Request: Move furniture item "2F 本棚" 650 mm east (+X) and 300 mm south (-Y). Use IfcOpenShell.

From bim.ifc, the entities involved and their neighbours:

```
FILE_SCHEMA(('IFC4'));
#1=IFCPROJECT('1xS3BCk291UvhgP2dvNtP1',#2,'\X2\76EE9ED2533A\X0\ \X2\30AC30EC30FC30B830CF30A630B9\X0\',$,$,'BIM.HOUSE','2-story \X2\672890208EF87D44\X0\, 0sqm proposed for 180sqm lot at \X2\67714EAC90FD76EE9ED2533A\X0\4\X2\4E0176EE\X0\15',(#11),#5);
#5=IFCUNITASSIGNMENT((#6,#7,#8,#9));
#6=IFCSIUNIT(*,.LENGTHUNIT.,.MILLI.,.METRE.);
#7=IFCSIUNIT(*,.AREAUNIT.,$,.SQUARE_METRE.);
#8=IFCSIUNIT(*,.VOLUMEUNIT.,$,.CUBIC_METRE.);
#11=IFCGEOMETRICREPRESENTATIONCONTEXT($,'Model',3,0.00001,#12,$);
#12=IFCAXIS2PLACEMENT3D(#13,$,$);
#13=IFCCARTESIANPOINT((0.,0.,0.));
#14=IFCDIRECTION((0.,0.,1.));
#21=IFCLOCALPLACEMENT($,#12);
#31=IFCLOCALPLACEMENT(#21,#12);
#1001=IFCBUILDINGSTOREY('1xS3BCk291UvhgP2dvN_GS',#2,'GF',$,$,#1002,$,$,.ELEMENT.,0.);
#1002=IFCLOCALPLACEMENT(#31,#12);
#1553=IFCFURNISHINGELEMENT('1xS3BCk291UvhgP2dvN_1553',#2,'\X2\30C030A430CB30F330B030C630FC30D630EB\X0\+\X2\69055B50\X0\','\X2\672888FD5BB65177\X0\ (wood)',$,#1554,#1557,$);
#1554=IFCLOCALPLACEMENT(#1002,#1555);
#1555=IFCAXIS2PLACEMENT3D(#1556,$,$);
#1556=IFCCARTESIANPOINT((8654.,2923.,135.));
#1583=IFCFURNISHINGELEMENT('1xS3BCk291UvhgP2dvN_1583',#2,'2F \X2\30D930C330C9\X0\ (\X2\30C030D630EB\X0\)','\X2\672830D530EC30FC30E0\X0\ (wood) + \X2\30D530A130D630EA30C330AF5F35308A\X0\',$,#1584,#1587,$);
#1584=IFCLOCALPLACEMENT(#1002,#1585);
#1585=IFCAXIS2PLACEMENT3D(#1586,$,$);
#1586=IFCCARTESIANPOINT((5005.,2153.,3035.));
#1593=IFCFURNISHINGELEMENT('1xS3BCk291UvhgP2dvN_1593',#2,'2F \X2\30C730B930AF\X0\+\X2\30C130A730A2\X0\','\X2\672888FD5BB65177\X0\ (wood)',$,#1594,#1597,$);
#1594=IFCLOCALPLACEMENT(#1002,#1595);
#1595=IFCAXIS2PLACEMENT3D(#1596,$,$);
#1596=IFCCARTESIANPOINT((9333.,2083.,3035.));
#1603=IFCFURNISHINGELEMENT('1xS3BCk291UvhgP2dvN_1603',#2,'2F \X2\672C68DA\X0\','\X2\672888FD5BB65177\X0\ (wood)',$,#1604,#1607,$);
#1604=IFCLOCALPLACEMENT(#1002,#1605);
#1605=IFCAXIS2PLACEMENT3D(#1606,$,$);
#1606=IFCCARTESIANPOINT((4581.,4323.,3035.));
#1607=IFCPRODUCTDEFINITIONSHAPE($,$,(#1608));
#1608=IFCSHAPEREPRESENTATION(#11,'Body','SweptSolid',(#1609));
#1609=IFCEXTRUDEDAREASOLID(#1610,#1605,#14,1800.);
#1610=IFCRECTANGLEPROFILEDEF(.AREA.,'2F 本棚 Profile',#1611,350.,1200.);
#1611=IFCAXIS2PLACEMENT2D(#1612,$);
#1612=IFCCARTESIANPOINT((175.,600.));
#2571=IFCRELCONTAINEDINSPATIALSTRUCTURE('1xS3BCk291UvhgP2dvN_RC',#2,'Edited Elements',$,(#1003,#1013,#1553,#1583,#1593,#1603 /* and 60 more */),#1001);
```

```python
import ifcopenshell
import ifcopenshell.api.geometry
import ifcopenshell.util.placement
import ifcopenshell.util.unit

model = ifcopenshell.open("bim.ifc")
unit_scale = ifcopenshell.util.unit.calculate_unit_scale(model)

item = model.by_guid("1xS3BCk291UvhgP2dvN_1603")
matrix = ifcopenshell.util.placement.get_local_placement(item.ObjectPlacement)
matrix[0, 3] += 0.65 / unit_scale
matrix[1, 3] -= 0.3 / unit_scale
ifcopenshell.api.geometry.edit_object_placement(model, product=item, matrix=matrix, is_si=False)

print(ifcopenshell.util.placement.get_local_placement(item.ObjectPlacement).round(3) + 0.0)

model.write("bim_rev.ifc")
```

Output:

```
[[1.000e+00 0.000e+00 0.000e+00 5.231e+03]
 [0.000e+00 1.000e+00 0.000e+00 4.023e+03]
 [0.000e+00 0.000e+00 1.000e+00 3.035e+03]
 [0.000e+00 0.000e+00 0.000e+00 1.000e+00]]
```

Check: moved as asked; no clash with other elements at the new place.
